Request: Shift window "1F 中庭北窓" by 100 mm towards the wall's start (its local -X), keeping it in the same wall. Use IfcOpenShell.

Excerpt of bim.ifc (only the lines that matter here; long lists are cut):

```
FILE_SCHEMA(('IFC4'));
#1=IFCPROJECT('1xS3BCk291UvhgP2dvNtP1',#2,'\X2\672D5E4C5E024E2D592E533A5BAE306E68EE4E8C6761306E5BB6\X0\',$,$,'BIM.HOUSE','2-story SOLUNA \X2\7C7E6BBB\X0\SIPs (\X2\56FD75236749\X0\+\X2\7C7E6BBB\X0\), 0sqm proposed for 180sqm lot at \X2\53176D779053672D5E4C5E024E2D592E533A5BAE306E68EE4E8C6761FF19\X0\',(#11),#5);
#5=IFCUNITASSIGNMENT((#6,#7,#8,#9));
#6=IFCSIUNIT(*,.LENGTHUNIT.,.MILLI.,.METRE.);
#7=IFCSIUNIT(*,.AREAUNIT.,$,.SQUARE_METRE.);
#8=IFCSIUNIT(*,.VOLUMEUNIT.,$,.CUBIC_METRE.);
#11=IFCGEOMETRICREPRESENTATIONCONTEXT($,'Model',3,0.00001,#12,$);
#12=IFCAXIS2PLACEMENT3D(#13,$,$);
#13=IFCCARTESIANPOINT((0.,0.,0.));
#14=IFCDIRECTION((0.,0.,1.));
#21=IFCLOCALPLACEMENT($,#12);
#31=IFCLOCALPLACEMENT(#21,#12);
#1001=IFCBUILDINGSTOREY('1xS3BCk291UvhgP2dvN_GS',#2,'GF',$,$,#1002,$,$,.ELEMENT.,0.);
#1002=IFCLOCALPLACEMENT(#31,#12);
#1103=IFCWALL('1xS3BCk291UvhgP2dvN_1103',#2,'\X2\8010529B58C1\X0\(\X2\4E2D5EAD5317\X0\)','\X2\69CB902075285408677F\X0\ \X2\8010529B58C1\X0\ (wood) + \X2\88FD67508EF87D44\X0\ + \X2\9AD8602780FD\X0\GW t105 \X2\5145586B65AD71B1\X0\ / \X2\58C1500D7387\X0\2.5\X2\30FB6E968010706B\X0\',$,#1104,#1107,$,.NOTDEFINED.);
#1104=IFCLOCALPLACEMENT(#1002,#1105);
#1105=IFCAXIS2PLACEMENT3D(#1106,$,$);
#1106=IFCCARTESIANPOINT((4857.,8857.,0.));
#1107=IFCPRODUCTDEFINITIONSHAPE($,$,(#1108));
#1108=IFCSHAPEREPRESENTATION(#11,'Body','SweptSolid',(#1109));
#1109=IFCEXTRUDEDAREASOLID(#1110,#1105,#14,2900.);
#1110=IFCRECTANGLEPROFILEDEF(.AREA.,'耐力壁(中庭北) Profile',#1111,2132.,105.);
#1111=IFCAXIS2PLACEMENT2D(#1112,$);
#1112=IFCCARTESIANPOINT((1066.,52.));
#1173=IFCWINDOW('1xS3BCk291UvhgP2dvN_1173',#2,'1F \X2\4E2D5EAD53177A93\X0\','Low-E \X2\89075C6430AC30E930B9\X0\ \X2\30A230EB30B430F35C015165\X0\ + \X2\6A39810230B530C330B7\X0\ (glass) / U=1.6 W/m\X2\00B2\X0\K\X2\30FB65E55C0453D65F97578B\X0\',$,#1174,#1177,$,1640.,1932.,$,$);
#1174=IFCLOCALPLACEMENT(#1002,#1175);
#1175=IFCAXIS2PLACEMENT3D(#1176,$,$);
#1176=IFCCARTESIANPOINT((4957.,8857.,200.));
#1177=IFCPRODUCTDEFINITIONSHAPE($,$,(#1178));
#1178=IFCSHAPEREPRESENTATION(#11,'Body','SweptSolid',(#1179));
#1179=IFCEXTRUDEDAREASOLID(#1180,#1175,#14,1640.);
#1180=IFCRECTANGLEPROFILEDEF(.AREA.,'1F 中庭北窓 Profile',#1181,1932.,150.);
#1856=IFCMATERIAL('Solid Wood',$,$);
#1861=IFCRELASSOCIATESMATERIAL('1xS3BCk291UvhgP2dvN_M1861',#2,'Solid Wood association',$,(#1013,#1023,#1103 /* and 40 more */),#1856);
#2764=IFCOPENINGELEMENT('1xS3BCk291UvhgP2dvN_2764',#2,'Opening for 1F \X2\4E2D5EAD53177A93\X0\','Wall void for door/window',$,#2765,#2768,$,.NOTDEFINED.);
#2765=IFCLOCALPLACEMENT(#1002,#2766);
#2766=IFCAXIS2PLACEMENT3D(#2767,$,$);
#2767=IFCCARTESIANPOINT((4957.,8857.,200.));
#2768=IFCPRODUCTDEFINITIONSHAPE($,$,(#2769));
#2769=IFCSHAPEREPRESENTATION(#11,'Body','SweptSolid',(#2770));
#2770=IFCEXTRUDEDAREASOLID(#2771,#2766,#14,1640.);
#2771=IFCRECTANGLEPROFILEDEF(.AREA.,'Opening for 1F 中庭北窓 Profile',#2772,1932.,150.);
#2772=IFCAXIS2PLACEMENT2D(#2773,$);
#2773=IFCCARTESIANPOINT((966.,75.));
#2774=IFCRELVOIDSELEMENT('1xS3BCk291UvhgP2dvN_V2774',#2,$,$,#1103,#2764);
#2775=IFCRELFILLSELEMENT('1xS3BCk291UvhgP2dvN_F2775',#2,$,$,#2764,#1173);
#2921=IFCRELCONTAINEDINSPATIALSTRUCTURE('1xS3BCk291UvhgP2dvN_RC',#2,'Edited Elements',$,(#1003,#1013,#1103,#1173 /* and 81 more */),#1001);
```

```python
import ifcopenshell
import ifcopenshell.api.geometry
import ifcopenshell.util.placement

model = ifcopenshell.open("bim.ifc")

window = model.by_guid("1xS3BCk291UvhgP2dvN_1173")
opening = window.FillsVoids[0].RelatingOpeningElement
wall = opening.VoidsElements[0].RelatingBuildingElement

wall_matrix = ifcopenshell.util.placement.get_local_placement(wall.ObjectPlacement)
shift = wall_matrix[:3, 0] * -100.0
before = ifcopenshell.util.placement.get_local_placement(window.ObjectPlacement)[:3, 3].copy()

# The window is not placed relative to its opening, so move both.
for product in (opening, window):
    matrix = ifcopenshell.util.placement.get_local_placement(product.ObjectPlacement)
    matrix[:3, 3] += shift
    ifcopenshell.api.geometry.edit_object_placement(model, product=product, matrix=matrix, is_si=False)

after = ifcopenshell.util.placement.get_local_placement(window.ObjectPlacement)[:3, 3]
print("window moved by", (after - before).round(3) + 0.0)

model.write("bim_v2.ifc")
```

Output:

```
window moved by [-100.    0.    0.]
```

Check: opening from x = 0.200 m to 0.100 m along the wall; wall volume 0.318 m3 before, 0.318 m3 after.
